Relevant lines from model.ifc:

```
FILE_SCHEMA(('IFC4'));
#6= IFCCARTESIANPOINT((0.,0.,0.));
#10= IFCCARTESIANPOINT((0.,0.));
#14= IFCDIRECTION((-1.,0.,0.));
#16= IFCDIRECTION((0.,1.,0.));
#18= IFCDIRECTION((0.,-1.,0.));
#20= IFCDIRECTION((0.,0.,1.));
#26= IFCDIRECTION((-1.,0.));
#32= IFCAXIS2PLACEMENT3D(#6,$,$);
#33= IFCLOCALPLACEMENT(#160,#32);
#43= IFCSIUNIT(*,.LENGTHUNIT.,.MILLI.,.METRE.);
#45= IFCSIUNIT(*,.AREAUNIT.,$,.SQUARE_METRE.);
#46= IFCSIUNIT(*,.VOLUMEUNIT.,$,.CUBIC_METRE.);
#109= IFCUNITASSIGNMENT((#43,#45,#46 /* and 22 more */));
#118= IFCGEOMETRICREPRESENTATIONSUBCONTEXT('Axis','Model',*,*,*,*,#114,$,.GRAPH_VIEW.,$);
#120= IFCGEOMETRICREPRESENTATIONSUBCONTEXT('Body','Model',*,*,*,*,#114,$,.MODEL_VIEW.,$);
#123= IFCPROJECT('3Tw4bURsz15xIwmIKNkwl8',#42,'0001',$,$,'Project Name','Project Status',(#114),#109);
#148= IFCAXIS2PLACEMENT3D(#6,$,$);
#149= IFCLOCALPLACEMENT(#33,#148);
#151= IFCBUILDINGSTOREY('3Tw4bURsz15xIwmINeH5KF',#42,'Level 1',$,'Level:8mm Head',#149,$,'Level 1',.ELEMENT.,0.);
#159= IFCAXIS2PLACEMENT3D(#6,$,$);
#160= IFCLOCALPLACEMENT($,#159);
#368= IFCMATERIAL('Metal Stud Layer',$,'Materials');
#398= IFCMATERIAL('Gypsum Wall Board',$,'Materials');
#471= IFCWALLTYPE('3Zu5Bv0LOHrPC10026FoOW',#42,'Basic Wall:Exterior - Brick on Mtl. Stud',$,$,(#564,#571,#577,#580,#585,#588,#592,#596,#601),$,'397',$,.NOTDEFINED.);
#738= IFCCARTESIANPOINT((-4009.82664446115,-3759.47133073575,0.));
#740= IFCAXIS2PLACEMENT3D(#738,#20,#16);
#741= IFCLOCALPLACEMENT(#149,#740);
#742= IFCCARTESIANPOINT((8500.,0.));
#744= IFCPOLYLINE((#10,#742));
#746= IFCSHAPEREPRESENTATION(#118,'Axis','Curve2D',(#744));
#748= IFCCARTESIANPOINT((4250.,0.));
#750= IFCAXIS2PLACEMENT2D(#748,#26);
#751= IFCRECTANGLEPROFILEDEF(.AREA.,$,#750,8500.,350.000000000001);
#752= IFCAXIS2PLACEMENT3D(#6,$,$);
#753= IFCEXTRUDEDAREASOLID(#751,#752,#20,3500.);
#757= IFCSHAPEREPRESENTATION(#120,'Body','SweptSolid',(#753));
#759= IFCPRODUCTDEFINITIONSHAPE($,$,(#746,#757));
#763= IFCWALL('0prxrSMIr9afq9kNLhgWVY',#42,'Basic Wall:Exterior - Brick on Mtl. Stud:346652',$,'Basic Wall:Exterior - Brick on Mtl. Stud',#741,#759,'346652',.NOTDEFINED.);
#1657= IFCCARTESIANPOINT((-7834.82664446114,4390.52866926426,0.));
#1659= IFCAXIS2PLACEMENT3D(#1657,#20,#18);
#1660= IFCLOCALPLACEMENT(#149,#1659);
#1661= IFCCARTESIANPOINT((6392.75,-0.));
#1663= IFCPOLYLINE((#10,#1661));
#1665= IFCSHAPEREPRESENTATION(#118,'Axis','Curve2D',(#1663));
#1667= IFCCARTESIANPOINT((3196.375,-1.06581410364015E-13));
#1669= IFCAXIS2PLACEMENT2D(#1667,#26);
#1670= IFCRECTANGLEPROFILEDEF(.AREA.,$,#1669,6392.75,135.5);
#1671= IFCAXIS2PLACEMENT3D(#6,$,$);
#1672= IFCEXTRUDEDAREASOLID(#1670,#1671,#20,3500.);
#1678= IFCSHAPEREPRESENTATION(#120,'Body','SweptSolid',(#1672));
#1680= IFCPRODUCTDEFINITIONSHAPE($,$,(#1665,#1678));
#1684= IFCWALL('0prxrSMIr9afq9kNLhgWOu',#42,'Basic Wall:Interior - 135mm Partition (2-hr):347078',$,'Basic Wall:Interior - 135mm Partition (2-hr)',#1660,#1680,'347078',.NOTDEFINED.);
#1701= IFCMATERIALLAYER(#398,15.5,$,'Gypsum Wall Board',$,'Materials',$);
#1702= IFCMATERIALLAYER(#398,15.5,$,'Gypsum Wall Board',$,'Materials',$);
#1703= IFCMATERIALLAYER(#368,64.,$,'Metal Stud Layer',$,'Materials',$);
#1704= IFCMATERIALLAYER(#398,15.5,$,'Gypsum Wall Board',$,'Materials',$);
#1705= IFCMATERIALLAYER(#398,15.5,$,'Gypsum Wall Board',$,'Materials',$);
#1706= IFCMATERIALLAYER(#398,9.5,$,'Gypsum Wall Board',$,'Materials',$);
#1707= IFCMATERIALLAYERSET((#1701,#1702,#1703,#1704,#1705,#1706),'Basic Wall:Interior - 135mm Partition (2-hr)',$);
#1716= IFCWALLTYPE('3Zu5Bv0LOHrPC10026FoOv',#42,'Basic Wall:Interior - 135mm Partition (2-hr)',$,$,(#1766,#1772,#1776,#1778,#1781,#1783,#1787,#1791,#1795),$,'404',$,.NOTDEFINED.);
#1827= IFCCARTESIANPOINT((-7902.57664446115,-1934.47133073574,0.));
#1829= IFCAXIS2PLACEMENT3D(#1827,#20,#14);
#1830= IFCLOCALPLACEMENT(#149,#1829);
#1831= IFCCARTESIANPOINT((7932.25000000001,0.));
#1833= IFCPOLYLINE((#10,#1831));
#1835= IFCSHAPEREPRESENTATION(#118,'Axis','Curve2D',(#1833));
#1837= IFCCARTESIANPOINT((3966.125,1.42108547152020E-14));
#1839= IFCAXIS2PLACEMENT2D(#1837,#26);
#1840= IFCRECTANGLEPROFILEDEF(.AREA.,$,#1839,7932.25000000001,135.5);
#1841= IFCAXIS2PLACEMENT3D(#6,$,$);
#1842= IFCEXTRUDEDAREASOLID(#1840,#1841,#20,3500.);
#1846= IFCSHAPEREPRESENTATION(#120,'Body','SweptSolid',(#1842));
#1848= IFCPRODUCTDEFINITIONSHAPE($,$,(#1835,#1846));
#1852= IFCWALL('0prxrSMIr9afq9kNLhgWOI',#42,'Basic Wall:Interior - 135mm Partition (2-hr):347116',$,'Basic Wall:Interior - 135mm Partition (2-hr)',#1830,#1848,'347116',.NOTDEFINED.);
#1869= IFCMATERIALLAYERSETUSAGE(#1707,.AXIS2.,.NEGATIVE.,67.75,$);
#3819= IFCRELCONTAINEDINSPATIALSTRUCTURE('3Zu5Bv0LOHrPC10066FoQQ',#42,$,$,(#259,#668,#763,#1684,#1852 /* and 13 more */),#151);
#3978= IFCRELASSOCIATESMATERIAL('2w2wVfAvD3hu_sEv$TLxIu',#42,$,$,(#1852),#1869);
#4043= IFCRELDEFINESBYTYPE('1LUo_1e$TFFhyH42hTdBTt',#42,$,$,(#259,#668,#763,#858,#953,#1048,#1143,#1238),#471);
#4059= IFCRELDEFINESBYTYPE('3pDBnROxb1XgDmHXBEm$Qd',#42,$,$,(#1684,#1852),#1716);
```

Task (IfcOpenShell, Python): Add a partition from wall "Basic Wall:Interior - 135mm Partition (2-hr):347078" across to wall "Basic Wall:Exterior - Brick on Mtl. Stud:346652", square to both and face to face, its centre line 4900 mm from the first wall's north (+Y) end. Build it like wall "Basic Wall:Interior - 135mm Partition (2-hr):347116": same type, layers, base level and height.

```python
import numpy as np
import ifcopenshell
import ifcopenshell.api.geometry
import ifcopenshell.api.material
import ifcopenshell.api.pset
import ifcopenshell.api.root
import ifcopenshell.api.spatial
import ifcopenshell.api.type
import ifcopenshell.geom
import ifcopenshell.util.element
import ifcopenshell.util.placement
import ifcopenshell.util.representation
import ifcopenshell.util.shape
import ifcopenshell.util.unit

model = ifcopenshell.open("model.ifc")
unit_scale = ifcopenshell.util.unit.calculate_unit_scale(model)
settings = ifcopenshell.geom.settings()
settings.set("use-world-coords", True)

start_wall = model.by_id(1684)
end_wall = model.by_guid("0prxrSMIr9afq9kNLhgWVY")
like = model.by_guid("0prxrSMIr9afq9kNLhgWOI")
matrix = ifcopenshell.util.placement.get_local_placement(start_wall.ObjectPlacement)
matrix[:3, 3] *= unit_scale


def extent(element):
    """Bounding box in the first wall's axes, in metres."""
    shape = ifcopenshell.geom.create_shape(settings, element)
    points = (ifcopenshell.util.shape.get_vertices(shape.geometry) - matrix[:3, 3]) @ matrix[:3, :3]
    return points.min(axis=0), points.max(axis=0)


y_start = extent(start_wall)[1][1]
y_end = extent(end_wall)[0][1]
like_min, like_max = extent(like)
length, height = float(abs(y_end - y_start)), float(like_max[2] - like_min[2])
layer_set = ifcopenshell.util.element.get_material(like, should_skip_usage=True)
thickness = sum(layer.LayerThickness for layer in layer_set.MaterialLayers) * unit_scale

wall = ifcopenshell.api.root.create_entity(model, ifc_class="IfcWall", name="New partition")
storey = ifcopenshell.util.element.get_container(like)
ifcopenshell.api.spatial.assign_container(model, products=[wall], relating_structure=storey)
ifcopenshell.api.type.assign_type(
    model, related_objects=[wall], relating_type=ifcopenshell.util.element.get_type(like), should_map_representations=False
)
rel = ifcopenshell.api.material.assign_material(
    model, products=[wall], type="IfcMaterialLayerSetUsage", material=layer_set
)
rel.RelatingMaterial.OffsetFromReferenceLine = -thickness / 2 / unit_scale
pset = ifcopenshell.api.pset.add_pset(model, product=wall, name="Pset_WallCommon")
ifcopenshell.api.pset.edit_pset(model, pset=pset, properties={"IsExternal": False, "LoadBearing": False})

# The axis runs down the middle of the wall.
axis = ifcopenshell.api.geometry.add_axis_representation(
    model, context=ifcopenshell.util.representation.get_context(model, "Model", "Axis"), axis=[(0.0, 0.0), (length, 0.0)]
)
body = ifcopenshell.api.geometry.add_wall_representation(
    model,
    context=ifcopenshell.util.representation.get_context(model, "Model", "Body", "MODEL_VIEW"),
    length=length,
    height=height,
    thickness=thickness,
    offset=-thickness / 2,
)
for representation in (axis, body):
    ifcopenshell.api.geometry.assign_representation(model, product=wall, representation=representation)

placement = matrix @ ifcopenshell.util.placement.rotation(90, "Z")
placement[:, 3] = matrix @ np.array([extent(start_wall)[0][0] + 4.9, y_start, like_min[2], 1.0])
ifcopenshell.api.geometry.edit_object_placement(model, product=wall, matrix=placement)

print(f"partition {length:.3f} m long, {height:.3f} m high, {thickness:.3f} m thick")

model.write("model-out.ifc")
```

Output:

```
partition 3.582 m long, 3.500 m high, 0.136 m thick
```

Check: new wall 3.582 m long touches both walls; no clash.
